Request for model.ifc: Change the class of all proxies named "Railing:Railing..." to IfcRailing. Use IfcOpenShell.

First a look at what the model holds.

```python
import re

import ifcopenshell

model = ifcopenshell.open("model.ifc")
print(model.schema)
seen = {}
for e in model.by_type("IfcBuildingElementProxy"):
    name = re.sub(r":\d+(:\d+)?$", "", e.Name or "")  # drop the element id that some exporters append
    seen[name] = seen.get(name, 0) + 1
for name, count in sorted(seen.items()):
    print(count, "x", name)
```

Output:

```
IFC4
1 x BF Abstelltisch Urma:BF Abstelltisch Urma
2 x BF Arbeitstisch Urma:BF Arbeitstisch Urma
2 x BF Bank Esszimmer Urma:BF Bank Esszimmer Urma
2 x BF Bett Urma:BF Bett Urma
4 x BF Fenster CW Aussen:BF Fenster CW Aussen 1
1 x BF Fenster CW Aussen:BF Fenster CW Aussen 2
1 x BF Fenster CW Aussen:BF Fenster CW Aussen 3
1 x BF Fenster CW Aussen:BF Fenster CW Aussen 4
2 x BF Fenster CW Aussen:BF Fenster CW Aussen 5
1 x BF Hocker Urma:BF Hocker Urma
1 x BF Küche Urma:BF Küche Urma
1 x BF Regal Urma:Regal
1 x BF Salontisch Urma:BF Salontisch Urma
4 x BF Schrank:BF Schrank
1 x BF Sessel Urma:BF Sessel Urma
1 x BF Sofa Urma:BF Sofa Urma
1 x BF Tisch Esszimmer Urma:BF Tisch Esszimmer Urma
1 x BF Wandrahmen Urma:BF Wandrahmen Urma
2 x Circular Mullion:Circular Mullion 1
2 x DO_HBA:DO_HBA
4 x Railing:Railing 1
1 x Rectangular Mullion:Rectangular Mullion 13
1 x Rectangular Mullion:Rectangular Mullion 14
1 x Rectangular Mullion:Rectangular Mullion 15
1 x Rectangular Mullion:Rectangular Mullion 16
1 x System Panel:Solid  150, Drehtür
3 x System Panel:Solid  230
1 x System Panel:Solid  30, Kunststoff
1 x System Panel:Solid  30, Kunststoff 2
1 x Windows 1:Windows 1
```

```python
import ifcopenshell
import ifcopenshell.api.root

model = ifcopenshell.open("model.ifc")

proxies = [e.id() for e in model.by_type("IfcBuildingElementProxy") if (e.Name or "").startswith("Railing:Railing")]
for step_id in proxies:
    proxy = model.by_id(step_id)
    ifcopenshell.api.root.reassign_class(model, product=proxy, ifc_class="IfcRailing")

print(sum(model.by_id(i).is_a("IfcRailing") for i in proxies), "reclassified")

model.write("model_updated.ifc")
```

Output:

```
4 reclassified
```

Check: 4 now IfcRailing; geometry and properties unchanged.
